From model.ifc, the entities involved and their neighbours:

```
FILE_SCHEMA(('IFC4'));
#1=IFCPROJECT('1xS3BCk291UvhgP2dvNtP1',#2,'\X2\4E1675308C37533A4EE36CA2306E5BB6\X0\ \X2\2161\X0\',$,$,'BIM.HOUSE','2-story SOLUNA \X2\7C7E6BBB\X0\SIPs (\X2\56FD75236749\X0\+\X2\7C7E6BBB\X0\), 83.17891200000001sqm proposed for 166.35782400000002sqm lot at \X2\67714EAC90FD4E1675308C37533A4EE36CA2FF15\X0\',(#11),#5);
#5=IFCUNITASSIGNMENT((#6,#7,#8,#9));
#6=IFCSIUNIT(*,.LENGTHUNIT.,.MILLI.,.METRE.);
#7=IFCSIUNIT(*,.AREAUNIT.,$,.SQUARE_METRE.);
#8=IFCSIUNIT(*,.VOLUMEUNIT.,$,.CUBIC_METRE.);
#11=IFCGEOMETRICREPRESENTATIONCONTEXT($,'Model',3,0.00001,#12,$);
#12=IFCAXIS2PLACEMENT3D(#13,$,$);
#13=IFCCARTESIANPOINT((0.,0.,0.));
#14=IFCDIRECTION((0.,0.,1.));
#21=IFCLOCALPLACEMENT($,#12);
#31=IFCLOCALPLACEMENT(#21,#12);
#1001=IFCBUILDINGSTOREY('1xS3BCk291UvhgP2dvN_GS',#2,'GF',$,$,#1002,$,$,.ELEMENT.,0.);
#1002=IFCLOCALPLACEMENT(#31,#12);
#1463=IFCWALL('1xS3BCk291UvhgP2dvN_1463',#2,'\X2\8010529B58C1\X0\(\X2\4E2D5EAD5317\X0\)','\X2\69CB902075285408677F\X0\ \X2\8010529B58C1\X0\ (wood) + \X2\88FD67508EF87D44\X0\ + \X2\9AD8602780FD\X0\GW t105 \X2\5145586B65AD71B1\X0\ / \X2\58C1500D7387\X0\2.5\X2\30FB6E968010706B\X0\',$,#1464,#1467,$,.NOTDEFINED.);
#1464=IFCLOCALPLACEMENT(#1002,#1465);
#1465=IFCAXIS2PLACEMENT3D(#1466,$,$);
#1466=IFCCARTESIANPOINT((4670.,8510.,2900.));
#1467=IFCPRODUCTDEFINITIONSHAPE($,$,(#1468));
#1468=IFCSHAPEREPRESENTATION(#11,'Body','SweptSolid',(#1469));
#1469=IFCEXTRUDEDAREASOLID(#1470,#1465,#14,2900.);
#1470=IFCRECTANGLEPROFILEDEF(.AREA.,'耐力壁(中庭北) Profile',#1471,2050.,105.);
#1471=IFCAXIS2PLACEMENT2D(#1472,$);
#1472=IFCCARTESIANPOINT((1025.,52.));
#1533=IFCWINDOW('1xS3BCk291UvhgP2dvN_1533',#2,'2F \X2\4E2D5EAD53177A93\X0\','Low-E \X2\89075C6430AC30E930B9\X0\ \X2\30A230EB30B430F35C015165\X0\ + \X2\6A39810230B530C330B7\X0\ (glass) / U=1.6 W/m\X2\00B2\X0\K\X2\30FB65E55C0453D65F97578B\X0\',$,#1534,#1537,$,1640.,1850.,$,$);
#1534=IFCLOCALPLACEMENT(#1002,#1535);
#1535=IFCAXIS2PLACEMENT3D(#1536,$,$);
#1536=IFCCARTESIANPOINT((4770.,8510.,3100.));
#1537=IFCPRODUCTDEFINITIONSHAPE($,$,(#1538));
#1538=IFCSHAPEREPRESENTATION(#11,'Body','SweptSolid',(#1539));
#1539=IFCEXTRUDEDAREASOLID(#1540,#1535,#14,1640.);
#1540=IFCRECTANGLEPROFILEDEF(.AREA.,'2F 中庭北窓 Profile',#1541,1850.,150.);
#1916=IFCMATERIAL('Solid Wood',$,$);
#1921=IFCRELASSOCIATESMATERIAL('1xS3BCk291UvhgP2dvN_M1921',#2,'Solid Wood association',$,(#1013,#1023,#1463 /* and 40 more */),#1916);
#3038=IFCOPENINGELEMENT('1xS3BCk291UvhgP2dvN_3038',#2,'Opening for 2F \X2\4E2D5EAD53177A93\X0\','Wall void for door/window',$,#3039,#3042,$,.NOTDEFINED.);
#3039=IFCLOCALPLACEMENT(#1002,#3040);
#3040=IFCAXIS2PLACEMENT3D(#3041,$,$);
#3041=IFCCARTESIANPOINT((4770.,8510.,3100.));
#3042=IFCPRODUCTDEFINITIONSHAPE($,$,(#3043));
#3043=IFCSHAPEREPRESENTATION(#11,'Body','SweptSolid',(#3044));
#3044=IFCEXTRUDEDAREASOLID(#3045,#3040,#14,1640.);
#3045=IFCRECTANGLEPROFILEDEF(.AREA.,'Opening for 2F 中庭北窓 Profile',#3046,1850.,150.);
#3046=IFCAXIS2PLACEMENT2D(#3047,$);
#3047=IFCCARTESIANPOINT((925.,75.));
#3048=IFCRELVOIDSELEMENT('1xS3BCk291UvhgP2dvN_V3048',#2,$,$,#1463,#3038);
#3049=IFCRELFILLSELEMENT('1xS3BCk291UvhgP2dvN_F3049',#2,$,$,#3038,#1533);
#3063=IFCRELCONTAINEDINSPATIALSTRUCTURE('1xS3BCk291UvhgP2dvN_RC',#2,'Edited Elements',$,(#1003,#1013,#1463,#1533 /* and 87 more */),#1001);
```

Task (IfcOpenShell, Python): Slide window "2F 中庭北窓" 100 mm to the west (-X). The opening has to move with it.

```python
import ifcopenshell
import ifcopenshell.api.geometry
import ifcopenshell.util.placement
import ifcopenshell.util.unit

model = ifcopenshell.open("model.ifc")
unit_scale = ifcopenshell.util.unit.calculate_unit_scale(model)

window = model.by_guid("1xS3BCk291UvhgP2dvN_1533")
opening = window.FillsVoids[0].RelatingOpeningElement
wall = opening.VoidsElements[0].RelatingBuildingElement

wall_matrix = ifcopenshell.util.placement.get_local_placement(wall.ObjectPlacement)
shift = wall_matrix[:3, 0] * -0.1 / unit_scale
before = ifcopenshell.util.placement.get_local_placement(window.ObjectPlacement)[:3, 3].copy()

# The window is not placed relative to its opening, so move both.
for product in (opening, window):
    matrix = ifcopenshell.util.placement.get_local_placement(product.ObjectPlacement)
    matrix[:3, 3] += shift
    ifcopenshell.api.geometry.edit_object_placement(model, product=product, matrix=matrix, is_si=False)

after = ifcopenshell.util.placement.get_local_placement(window.ObjectPlacement)[:3, 3]
print("window moved by", (after - before).round(3) + 0.0)

model.write("model_edited.ifc")
```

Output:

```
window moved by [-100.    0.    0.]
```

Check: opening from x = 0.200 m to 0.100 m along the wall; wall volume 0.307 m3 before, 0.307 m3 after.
